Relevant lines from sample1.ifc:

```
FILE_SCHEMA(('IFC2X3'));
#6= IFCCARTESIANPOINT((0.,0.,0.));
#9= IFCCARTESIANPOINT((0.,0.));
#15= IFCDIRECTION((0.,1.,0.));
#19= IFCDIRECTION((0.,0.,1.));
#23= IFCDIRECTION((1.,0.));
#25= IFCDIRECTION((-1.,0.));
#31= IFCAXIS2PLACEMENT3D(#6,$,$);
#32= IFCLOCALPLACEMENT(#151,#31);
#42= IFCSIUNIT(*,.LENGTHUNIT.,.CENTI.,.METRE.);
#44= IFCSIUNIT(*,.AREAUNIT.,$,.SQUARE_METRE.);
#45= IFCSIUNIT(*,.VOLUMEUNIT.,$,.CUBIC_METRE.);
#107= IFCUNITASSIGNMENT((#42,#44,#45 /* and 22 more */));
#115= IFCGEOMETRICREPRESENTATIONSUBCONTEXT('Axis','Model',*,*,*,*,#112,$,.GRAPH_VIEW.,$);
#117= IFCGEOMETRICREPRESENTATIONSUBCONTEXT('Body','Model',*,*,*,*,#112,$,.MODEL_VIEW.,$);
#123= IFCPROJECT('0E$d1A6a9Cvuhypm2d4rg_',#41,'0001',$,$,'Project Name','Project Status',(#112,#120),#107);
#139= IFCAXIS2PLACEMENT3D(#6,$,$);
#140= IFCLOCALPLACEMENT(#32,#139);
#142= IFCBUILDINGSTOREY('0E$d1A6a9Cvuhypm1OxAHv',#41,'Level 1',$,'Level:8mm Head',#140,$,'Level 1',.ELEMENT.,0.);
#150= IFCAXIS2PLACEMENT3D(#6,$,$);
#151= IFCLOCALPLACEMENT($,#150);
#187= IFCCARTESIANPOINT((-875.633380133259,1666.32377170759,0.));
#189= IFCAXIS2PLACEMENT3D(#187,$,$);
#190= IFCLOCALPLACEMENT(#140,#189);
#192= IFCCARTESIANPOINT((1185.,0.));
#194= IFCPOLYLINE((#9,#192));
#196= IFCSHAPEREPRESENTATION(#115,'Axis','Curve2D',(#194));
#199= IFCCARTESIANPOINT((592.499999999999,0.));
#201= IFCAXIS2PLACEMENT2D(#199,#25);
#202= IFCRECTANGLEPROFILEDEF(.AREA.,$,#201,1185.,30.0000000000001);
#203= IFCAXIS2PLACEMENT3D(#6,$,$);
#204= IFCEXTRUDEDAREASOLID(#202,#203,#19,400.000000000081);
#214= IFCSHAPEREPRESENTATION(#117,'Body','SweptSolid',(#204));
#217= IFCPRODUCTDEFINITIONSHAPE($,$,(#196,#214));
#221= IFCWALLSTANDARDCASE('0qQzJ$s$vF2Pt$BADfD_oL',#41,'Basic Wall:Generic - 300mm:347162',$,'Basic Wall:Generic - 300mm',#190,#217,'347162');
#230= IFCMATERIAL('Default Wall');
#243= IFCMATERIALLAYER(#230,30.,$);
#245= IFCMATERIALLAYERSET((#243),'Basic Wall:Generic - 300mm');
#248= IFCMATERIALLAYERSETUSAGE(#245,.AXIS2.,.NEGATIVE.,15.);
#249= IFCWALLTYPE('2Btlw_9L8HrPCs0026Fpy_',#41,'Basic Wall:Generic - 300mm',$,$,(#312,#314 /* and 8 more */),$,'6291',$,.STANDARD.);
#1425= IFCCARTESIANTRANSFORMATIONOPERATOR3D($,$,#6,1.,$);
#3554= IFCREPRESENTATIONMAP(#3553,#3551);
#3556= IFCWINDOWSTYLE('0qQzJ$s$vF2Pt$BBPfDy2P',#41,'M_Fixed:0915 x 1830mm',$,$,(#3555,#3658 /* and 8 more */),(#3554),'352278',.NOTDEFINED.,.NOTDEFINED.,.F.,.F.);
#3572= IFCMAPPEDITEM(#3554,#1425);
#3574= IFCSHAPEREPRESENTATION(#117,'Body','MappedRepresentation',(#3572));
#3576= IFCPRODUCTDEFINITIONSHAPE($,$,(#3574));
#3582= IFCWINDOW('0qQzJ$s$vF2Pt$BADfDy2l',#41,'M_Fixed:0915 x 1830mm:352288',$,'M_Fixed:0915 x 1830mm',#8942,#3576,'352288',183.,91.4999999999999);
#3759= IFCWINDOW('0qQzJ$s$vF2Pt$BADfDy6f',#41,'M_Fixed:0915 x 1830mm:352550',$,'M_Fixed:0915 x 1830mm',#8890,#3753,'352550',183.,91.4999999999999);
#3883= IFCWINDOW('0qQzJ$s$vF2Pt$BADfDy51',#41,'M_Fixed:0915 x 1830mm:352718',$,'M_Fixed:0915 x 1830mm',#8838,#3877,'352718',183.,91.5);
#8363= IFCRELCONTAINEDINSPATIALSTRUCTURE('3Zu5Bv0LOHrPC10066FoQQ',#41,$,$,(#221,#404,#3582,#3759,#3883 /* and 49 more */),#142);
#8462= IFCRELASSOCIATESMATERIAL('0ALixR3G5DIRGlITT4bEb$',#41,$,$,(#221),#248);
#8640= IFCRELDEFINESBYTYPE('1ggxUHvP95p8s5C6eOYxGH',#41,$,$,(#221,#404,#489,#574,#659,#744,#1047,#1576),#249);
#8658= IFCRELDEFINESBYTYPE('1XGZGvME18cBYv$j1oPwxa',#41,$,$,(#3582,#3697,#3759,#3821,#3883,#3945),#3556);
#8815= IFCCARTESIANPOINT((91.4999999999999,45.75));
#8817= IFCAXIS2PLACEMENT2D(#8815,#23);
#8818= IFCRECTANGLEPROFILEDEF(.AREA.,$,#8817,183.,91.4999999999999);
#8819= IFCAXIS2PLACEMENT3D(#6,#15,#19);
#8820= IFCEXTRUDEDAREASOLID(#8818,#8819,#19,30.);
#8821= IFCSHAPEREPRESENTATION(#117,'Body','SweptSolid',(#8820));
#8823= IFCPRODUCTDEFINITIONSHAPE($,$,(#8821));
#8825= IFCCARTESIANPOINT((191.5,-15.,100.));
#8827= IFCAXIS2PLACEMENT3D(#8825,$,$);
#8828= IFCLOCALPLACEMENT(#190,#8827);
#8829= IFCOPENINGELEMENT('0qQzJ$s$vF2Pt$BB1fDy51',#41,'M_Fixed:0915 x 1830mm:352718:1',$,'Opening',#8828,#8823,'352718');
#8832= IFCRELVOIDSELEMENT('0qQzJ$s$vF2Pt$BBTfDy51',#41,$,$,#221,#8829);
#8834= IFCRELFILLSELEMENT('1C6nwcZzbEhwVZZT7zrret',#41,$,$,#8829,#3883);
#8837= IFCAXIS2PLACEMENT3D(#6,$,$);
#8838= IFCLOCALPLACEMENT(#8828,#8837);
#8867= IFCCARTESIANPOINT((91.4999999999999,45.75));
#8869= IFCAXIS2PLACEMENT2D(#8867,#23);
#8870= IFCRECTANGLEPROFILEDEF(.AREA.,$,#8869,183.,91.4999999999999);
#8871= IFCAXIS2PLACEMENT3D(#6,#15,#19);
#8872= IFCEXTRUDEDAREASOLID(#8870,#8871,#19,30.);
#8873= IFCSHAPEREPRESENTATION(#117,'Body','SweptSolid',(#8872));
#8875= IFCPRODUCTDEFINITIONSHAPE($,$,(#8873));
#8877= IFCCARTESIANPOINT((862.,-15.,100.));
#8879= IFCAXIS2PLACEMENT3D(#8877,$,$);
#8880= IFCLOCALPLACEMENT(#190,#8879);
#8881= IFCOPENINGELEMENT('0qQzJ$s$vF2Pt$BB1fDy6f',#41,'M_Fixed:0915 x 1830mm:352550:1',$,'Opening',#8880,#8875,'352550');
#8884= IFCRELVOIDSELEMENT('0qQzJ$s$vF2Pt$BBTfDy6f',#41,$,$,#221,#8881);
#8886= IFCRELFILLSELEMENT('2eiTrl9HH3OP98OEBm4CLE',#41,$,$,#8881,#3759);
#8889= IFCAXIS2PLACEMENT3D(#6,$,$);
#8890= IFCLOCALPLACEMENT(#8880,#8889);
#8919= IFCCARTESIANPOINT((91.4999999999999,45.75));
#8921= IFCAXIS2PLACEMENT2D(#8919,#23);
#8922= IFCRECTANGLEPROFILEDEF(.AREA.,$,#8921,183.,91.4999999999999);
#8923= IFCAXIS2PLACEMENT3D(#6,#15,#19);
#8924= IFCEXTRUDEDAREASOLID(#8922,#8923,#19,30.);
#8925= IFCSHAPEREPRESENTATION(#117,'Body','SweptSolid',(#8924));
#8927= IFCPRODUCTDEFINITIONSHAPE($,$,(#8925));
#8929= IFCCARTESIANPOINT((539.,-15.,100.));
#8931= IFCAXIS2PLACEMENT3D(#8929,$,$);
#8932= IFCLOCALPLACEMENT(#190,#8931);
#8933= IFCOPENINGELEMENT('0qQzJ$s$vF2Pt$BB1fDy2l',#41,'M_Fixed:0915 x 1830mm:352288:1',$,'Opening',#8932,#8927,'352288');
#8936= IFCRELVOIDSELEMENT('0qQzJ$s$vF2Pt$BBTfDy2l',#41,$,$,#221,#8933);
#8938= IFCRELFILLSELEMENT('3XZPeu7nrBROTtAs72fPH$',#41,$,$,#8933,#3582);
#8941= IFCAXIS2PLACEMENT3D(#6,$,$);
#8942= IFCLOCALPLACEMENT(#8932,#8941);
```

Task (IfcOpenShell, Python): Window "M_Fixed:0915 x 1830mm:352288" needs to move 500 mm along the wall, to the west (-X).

```python
import ifcopenshell
import ifcopenshell.api.geometry
import ifcopenshell.util.placement
import ifcopenshell.util.unit

model = ifcopenshell.open("sample1.ifc")
unit_scale = ifcopenshell.util.unit.calculate_unit_scale(model)

window = model.by_guid("0qQzJ$s$vF2Pt$BADfDy2l")
opening = window.FillsVoids[0].RelatingOpeningElement
wall = opening.VoidsElements[0].RelatingBuildingElement

wall_matrix = ifcopenshell.util.placement.get_local_placement(wall.ObjectPlacement)
shift = wall_matrix[:3, 0] * -0.5 / unit_scale
before = ifcopenshell.util.placement.get_local_placement(window.ObjectPlacement)[:3, 3].copy()

# The window is placed relative to its opening, so it follows when the opening moves.
matrix = ifcopenshell.util.placement.get_local_placement(opening.ObjectPlacement)
matrix[:3, 3] += shift
ifcopenshell.api.geometry.edit_object_placement(
    model, product=opening, matrix=matrix, is_si=False, should_transform_children=True
)

after = ifcopenshell.util.placement.get_local_placement(window.ObjectPlacement)[:3, 3]
print("window moved by", (after - before).round(3) + 0.0)

model.write("sample1_edited.ifc")
```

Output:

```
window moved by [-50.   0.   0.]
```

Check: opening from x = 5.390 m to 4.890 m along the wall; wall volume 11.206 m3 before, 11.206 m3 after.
